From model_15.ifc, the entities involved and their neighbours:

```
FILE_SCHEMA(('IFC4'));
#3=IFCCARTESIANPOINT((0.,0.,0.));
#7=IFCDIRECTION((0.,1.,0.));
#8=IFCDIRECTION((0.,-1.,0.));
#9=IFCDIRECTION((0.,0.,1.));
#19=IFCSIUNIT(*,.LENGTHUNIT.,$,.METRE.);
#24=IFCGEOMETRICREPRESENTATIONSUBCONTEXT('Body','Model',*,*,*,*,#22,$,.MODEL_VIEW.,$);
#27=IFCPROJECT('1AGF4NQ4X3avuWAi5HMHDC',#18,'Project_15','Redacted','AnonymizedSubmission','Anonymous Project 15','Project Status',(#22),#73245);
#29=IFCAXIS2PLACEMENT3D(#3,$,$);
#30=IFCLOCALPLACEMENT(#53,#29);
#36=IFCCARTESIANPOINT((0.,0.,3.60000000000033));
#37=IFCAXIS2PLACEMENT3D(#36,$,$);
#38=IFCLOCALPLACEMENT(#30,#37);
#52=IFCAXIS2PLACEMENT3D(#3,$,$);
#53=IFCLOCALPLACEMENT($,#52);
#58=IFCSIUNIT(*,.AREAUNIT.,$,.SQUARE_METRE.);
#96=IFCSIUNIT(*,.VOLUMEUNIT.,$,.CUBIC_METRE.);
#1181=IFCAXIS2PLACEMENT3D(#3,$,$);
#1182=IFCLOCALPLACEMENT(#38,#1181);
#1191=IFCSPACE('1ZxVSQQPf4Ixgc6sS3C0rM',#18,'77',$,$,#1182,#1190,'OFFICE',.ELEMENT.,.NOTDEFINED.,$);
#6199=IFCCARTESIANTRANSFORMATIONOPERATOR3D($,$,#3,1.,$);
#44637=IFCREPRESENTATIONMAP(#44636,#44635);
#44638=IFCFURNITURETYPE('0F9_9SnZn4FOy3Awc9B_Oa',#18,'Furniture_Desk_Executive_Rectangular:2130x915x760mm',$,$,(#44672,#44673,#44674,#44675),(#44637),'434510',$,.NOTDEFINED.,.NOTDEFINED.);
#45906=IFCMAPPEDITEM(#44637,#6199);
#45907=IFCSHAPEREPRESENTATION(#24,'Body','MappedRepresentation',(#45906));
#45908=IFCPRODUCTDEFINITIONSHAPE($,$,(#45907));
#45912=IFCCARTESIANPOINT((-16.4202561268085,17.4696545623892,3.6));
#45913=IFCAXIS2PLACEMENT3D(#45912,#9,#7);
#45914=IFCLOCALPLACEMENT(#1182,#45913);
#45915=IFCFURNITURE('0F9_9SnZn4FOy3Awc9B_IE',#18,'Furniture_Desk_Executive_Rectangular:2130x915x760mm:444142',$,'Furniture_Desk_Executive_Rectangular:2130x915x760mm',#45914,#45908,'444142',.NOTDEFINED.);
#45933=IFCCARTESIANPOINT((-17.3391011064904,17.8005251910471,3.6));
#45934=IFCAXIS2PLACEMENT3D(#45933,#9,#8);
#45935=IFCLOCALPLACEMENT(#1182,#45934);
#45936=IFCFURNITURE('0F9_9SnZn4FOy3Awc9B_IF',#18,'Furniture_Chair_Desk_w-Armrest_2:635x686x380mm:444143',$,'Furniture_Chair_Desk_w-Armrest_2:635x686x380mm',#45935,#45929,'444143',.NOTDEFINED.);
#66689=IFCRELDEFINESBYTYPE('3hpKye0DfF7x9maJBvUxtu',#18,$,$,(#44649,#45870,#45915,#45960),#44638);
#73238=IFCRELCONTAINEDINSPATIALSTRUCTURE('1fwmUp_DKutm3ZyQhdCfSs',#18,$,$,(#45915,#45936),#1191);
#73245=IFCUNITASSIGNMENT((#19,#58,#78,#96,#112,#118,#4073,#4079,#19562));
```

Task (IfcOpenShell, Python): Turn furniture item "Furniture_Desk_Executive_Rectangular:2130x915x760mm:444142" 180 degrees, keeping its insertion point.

```python
import ifcopenshell
import ifcopenshell.api.geometry
import ifcopenshell.util.placement

model = ifcopenshell.open("model_15.ifc")

item = model.by_id(45915)
matrix = ifcopenshell.util.placement.get_local_placement(item.ObjectPlacement)
matrix = matrix @ ifcopenshell.util.placement.rotation(180, "Z")
ifcopenshell.api.geometry.edit_object_placement(model, product=item, matrix=matrix, is_si=False)

print(ifcopenshell.util.placement.get_local_placement(item.ObjectPlacement).round(3) + 0.0)

model.write("model_15-out.ifc")
```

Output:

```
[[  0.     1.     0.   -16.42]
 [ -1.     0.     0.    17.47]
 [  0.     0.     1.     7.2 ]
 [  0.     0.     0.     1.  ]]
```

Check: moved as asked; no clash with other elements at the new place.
